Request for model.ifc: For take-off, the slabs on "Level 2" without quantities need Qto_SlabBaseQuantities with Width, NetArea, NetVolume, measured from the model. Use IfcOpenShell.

First a look at what the model holds.

```python
import ifcopenshell
import ifcopenshell.util.element
import ifcopenshell.util.unit

model = ifcopenshell.open("model.ifc")
print(model.schema)
for unit_type in ("LENGTHUNIT", "AREAUNIT", "VOLUMEUNIT"):
    print(unit_type, ifcopenshell.util.unit.calculate_unit_scale(model, unit_type))
storey = next(s for s in model.by_type("IfcBuildingStorey") if s.Name == "Level 2")
slabs = [e for e in ifcopenshell.util.element.get_decomposition(storey) if e.is_a("IfcSlab")]
for e in sorted(slabs, key=lambda e: e.id()):
    print(e.id(), e.is_a(), e.Name, list(ifcopenshell.util.element.get_psets(e, qtos_only=True)), sep=" | ")
```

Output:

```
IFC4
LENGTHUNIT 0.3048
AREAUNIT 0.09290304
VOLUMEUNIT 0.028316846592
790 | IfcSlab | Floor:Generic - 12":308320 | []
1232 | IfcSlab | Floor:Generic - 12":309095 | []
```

```python
import ifcopenshell
import ifcopenshell.api.pset
import ifcopenshell.geom
import ifcopenshell.util.element
import ifcopenshell.util.shape
import ifcopenshell.util.unit

model = ifcopenshell.open("model.ifc")
unit_scale = ifcopenshell.util.unit.calculate_unit_scale(model)
area_scale = ifcopenshell.util.unit.calculate_unit_scale(model, "AREAUNIT")
volume_scale = ifcopenshell.util.unit.calculate_unit_scale(model, "VOLUMEUNIT")
settings = ifcopenshell.geom.settings()

storey = next(s for s in model.by_type("IfcBuildingStorey") if s.Name == "Level 2")
slabs = [e for e in ifcopenshell.util.element.get_decomposition(storey) if e.is_a("IfcSlab")]

for e in sorted(slabs, key=lambda e: e.id()):
    if ifcopenshell.util.element.get_psets(e, qtos_only=True, should_inherit=False):
        continue
    # Geometry comes back in metres, in the element's own axes.
    shape = ifcopenshell.geom.create_shape(settings, e)
    values = {
        "Width": ifcopenshell.util.shape.get_z(shape.geometry) / unit_scale,
        "NetArea": ifcopenshell.util.shape.get_footprint_area(shape.geometry) / area_scale,
        "NetVolume": ifcopenshell.util.shape.get_volume(shape.geometry) / volume_scale,
    }
    qto = ifcopenshell.api.pset.add_qto(model, product=e, name="Qto_SlabBaseQuantities")
    ifcopenshell.api.pset.edit_qto(model, qto=qto, properties=values)
    print(e.id(), {k: round(v, 3) for k, v in values.items()})

model.write("model_edited.ifc")
```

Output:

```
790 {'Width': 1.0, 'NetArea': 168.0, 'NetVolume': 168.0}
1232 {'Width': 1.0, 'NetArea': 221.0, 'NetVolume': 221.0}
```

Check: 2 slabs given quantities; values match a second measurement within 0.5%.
